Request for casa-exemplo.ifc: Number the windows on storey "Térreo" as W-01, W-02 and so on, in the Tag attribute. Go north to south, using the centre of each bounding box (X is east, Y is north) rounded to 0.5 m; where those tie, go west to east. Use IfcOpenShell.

First a look at what the model holds.

```python
import ifcopenshell
import ifcopenshell.util.element
import ifcopenshell.util.placement

model = ifcopenshell.open("casa-exemplo.ifc")
print(model.schema)
storey = next(s for s in model.by_type("IfcBuildingStorey") if s.Name == "Térreo")
windows = [e for e in ifcopenshell.util.element.get_decomposition(storey) if e.is_a("IfcWindow")]
for e in sorted(windows, key=lambda e: e.id()):
    origin = ifcopenshell.util.placement.get_local_placement(e.ObjectPlacement)[:3, 3]
    print(e.id(), e.Tag, e.Name, origin.round(2) + 0.0, sep=" | ")
```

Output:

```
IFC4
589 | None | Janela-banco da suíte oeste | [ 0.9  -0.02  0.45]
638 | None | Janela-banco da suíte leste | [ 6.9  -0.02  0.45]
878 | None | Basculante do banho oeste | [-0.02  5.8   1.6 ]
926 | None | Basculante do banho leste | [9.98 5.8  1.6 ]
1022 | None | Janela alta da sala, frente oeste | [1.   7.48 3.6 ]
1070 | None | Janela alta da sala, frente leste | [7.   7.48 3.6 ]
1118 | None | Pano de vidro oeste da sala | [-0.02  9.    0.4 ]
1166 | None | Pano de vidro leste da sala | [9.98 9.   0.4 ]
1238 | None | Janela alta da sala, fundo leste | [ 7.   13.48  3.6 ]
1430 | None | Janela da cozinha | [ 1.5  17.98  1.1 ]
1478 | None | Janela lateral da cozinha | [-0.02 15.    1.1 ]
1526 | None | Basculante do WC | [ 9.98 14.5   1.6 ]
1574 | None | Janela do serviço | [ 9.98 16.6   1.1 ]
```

```python
import ifcopenshell
import ifcopenshell.geom
import ifcopenshell.util.element
import ifcopenshell.util.shape

model = ifcopenshell.open("casa-exemplo.ifc")
settings = ifcopenshell.geom.settings()
settings.set("use-world-coords", True)


def centre(element):
    shape = ifcopenshell.geom.create_shape(settings, element)
    return ifcopenshell.util.shape.get_bbox_centroid(shape.geometry)


storey = next(s for s in model.by_type("IfcBuildingStorey") if s.Name == "Térreo")
windows = [e for e in ifcopenshell.util.element.get_decomposition(storey) if e.is_a("IfcWindow")]

# Insertion points can sit at a corner or the storey origin, so sort by the geometry (in metres).
centres = {e: centre(e) for e in windows}
windows.sort(key=lambda e: (-round(centres[e][1] / 0.5), centres[e][0]))

for i, e in enumerate(windows, start=1):
    number = f"W-{i:02d}"
    e.Tag = number
    print(e.id(), number)

model.write("casa-exemplo_updated.ifc")
```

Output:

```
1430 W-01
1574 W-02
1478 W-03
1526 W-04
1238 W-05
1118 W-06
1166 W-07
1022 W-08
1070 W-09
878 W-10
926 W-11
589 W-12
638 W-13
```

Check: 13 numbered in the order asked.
